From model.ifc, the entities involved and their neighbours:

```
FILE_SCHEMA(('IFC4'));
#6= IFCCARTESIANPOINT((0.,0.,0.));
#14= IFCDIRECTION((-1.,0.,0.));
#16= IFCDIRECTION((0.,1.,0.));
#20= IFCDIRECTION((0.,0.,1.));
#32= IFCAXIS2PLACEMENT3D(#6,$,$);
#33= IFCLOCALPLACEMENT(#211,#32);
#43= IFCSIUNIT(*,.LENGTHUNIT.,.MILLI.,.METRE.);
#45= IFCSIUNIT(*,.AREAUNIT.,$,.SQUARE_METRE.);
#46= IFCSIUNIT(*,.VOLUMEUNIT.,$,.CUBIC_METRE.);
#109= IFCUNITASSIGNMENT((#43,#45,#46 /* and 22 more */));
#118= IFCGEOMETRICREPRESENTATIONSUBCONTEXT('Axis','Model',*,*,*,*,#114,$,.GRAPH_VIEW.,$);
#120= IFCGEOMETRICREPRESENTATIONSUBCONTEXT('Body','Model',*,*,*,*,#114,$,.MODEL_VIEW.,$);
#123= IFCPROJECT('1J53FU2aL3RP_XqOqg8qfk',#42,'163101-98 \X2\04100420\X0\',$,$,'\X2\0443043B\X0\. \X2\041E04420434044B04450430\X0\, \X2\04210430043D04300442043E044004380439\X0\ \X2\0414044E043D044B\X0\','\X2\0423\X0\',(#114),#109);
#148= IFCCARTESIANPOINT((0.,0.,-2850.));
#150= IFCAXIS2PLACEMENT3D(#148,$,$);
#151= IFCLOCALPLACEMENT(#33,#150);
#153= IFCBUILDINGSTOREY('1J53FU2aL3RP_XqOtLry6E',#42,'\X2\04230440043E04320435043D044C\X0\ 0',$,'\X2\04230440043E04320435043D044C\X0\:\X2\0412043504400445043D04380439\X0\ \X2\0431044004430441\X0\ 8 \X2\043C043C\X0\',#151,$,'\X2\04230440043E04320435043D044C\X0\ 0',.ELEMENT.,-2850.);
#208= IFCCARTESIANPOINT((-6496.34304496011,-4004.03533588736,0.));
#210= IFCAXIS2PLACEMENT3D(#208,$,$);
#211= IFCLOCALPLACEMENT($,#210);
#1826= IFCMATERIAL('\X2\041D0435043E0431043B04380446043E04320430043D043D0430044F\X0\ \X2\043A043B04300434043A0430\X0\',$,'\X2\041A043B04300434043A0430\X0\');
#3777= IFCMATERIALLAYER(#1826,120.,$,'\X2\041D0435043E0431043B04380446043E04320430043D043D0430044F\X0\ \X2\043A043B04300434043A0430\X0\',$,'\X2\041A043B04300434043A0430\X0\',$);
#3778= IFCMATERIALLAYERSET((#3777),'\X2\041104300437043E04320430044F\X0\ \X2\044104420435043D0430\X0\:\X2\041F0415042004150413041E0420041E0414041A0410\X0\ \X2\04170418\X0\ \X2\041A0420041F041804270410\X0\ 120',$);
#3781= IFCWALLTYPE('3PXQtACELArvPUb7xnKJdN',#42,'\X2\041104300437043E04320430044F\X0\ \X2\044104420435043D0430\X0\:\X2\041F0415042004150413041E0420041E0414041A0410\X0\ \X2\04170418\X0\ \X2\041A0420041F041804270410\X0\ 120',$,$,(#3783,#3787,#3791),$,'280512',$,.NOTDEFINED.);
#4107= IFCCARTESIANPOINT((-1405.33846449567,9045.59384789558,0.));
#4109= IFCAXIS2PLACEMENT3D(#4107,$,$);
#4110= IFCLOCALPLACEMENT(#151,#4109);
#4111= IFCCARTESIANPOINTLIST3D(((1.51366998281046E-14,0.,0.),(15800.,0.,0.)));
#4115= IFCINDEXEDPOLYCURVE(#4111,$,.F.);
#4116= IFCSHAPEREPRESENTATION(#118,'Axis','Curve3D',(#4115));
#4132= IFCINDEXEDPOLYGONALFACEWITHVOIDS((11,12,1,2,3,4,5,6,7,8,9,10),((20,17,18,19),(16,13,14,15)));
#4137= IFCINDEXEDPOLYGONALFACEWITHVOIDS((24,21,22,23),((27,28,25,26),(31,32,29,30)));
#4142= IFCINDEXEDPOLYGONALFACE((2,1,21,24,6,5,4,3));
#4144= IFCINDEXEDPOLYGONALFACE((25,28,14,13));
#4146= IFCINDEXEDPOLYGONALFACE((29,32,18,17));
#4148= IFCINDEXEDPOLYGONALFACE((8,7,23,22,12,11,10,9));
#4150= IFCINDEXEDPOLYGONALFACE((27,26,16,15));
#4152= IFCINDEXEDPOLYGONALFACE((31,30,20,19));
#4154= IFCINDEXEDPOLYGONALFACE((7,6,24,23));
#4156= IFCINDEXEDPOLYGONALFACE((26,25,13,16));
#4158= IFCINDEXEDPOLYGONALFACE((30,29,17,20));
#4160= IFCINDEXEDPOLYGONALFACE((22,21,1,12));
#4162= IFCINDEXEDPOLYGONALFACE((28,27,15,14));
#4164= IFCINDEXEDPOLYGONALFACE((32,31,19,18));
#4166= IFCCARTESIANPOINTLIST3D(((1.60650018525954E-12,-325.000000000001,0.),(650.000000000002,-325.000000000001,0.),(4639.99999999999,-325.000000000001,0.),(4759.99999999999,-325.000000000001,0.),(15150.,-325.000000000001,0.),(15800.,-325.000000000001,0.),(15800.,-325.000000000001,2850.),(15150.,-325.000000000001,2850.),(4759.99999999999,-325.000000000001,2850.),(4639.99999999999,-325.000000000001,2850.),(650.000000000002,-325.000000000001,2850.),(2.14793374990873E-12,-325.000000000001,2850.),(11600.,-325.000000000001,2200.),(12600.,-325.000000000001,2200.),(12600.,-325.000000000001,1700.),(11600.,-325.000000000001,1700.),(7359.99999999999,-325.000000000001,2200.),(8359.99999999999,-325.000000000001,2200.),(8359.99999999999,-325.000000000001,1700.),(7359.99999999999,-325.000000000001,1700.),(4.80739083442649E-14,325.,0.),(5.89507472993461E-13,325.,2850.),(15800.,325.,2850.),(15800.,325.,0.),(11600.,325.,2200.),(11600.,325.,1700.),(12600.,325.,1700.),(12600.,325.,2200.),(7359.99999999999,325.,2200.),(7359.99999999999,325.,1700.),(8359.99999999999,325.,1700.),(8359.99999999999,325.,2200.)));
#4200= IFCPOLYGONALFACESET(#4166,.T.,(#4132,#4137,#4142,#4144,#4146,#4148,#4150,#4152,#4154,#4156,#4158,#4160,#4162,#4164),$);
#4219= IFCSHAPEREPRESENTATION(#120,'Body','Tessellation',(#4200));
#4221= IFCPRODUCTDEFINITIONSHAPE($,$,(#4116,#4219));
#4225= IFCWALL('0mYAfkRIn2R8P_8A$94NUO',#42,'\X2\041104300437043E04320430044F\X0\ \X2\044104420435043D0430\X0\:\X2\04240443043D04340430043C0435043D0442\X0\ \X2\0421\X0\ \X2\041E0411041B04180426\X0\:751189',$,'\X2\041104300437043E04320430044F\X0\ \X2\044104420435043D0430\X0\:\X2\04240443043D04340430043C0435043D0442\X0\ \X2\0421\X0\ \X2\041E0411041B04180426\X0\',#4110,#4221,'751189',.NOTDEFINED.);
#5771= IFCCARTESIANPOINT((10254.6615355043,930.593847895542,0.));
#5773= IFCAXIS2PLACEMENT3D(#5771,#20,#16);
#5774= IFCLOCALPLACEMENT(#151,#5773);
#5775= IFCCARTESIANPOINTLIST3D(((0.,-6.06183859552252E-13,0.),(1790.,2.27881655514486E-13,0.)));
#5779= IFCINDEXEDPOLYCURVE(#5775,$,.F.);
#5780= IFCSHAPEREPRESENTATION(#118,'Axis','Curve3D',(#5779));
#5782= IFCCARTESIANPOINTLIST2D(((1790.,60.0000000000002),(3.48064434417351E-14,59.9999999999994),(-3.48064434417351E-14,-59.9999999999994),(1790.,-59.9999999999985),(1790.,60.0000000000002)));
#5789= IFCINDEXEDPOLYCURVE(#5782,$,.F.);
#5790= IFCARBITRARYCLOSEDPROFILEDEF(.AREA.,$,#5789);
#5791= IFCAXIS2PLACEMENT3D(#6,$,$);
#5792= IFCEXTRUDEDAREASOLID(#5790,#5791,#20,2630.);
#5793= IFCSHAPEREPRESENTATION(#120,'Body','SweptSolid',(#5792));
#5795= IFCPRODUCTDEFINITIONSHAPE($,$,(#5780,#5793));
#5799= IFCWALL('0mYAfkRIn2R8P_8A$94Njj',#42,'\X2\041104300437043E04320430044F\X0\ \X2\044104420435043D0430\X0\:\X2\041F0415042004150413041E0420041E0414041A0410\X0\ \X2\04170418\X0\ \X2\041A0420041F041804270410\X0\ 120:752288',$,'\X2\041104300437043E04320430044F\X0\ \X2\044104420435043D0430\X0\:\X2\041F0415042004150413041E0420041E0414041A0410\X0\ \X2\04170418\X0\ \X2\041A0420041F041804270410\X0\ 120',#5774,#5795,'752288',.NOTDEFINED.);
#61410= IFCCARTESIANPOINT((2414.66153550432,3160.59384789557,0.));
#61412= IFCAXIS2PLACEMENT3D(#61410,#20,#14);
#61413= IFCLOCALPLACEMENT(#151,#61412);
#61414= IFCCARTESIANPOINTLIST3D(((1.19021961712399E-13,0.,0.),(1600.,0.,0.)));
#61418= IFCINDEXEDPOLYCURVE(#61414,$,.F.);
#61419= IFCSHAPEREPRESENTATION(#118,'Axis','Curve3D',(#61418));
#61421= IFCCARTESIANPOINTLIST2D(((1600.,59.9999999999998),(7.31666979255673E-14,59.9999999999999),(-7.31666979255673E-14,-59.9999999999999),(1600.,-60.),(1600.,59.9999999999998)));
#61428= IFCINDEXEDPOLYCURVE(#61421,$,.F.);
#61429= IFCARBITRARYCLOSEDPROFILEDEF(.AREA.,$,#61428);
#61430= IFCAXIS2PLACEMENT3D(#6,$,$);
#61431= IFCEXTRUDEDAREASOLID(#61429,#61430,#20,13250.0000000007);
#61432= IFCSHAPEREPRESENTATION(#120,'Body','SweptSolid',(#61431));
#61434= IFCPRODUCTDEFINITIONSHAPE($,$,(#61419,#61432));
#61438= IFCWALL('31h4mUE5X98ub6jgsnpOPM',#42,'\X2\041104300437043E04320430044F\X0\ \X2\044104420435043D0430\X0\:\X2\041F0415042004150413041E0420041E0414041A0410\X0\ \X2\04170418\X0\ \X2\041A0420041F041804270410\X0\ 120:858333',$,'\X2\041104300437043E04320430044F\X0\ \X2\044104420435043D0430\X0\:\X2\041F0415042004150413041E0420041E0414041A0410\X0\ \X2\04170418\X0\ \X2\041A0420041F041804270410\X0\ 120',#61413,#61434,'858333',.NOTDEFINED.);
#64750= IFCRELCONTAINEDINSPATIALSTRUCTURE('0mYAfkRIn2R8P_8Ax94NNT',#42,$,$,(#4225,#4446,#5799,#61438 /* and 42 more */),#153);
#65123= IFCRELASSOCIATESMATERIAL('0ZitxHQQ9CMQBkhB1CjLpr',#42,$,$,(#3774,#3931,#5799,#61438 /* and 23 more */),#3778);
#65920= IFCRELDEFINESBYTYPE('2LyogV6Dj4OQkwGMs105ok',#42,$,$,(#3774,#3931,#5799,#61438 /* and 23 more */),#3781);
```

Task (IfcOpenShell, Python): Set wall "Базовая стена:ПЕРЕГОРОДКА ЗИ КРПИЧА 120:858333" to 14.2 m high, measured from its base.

```python
import ifcopenshell
import ifcopenshell.geom
import ifcopenshell.util.representation
import ifcopenshell.util.shape
import ifcopenshell.util.unit

model = ifcopenshell.open("model.ifc")
unit_scale = ifcopenshell.util.unit.calculate_unit_scale(model)
settings = ifcopenshell.geom.settings()


def volume(element):
    """Net volume in cubic metres, openings subtracted."""
    shape = ifcopenshell.geom.create_shape(settings, element)
    return ifcopenshell.util.shape.get_volume(shape.geometry)


wall = model.by_guid("31h4mUE5X98ub6jgsnpOPM")
before = volume(wall)

body = ifcopenshell.util.representation.get_representation(wall, "Model", "Body")
solid = body.Items[0]
old_height = solid.Depth
solid.Depth = 14.2 / unit_scale
after = volume(wall)

print(f"height {old_height:g} -> {solid.Depth:g}, volume {before:.3f} -> {after:.3f} m3")

model.write("model_updated.ifc")
```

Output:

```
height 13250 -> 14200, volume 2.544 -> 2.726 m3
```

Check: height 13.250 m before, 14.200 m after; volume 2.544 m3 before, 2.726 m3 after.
